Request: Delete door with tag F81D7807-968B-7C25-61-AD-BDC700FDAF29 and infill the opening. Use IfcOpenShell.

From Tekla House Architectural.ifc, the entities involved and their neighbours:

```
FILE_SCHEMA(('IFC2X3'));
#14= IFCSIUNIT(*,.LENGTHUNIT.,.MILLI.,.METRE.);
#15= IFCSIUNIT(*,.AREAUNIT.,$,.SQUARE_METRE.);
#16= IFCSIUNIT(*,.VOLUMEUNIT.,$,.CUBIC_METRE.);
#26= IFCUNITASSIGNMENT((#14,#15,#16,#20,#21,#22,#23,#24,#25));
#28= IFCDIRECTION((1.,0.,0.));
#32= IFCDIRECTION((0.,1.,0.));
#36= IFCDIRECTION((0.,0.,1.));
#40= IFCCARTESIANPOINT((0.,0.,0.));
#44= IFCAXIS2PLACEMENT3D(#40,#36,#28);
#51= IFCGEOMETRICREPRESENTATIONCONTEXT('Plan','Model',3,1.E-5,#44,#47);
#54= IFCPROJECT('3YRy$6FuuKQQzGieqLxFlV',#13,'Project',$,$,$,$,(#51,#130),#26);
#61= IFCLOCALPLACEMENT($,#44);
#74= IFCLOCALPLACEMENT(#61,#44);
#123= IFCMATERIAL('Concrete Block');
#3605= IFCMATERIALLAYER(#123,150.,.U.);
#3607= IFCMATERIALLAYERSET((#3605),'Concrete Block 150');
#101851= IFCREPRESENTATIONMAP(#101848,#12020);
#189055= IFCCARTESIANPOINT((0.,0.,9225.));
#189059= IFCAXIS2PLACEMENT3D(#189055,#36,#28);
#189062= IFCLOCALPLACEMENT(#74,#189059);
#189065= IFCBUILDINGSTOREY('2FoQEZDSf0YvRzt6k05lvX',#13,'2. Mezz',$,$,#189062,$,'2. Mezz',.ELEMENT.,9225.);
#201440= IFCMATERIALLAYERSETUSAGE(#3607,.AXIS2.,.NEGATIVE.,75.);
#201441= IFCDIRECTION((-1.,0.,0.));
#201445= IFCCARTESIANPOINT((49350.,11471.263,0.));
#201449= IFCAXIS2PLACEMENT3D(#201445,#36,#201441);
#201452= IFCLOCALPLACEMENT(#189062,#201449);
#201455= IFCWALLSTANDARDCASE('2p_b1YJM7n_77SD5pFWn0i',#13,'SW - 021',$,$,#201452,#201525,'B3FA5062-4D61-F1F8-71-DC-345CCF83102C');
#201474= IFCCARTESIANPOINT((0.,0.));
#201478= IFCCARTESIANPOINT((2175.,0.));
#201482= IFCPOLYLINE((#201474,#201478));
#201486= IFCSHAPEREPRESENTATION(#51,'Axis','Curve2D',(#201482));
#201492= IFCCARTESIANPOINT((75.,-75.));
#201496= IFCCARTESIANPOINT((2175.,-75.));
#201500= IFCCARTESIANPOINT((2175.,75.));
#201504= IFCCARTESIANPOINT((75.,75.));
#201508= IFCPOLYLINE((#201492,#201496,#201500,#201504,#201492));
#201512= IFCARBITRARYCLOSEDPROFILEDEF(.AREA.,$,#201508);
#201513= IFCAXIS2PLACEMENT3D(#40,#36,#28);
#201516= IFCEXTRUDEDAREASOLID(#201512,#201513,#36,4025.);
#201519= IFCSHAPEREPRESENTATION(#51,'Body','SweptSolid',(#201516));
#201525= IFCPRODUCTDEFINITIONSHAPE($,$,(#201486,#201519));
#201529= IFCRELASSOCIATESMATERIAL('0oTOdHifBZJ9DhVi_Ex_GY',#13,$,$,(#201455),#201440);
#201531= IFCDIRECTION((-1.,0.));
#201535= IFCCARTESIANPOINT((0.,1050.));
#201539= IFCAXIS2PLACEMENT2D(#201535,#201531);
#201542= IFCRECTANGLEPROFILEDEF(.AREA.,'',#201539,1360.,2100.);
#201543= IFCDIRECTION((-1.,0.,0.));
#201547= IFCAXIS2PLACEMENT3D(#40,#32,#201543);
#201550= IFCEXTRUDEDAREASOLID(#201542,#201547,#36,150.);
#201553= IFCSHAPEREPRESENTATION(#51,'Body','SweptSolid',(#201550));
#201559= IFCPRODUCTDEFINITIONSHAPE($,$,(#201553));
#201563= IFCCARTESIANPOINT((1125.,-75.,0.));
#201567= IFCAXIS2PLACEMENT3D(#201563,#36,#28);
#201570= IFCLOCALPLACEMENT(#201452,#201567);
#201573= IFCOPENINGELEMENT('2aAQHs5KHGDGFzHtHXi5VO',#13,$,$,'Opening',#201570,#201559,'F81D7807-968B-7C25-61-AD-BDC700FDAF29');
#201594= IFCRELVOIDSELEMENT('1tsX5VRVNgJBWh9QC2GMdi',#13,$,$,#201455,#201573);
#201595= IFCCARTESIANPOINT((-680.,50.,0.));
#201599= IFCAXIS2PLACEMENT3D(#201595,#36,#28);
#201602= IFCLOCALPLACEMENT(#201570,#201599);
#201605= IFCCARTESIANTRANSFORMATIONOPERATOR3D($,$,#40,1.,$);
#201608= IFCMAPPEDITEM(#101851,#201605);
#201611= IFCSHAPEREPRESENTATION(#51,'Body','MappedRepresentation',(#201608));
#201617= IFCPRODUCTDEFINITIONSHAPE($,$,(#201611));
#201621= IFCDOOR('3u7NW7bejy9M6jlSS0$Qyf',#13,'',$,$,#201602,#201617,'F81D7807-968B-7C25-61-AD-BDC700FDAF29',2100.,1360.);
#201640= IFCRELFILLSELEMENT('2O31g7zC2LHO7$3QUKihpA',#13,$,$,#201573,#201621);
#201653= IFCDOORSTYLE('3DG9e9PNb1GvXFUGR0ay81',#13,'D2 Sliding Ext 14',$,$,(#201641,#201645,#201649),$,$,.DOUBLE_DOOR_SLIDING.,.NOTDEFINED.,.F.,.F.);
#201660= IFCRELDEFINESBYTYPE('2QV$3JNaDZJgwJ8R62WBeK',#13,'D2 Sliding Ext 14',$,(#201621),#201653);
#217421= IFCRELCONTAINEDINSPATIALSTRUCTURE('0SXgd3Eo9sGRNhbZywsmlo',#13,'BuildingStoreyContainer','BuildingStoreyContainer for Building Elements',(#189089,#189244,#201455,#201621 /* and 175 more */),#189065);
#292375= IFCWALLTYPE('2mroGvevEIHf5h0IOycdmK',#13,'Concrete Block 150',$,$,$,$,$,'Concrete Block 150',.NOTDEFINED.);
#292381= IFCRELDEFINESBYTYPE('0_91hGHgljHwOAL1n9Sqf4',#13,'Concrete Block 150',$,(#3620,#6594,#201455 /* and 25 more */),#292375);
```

```python
import ifcopenshell
import ifcopenshell.api.feature
import ifcopenshell.api.root
import ifcopenshell.geom
import ifcopenshell.util.shape

model = ifcopenshell.open("Tekla House Architectural.ifc")
settings = ifcopenshell.geom.settings()


def volume(element):
    """Net volume in cubic metres, openings subtracted."""
    shape = ifcopenshell.geom.create_shape(settings, element)
    return ifcopenshell.util.shape.get_volume(shape.geometry)


door = model.by_guid("3u7NW7bejy9M6jlSS0$Qyf")
opening = door.FillsVoids[0].RelatingOpeningElement
wall = opening.VoidsElements[0].RelatingBuildingElement
before = volume(wall)

ifcopenshell.api.root.remove_product(model, product=door)
ifcopenshell.api.feature.remove_feature(model, feature=opening)

after = volume(wall)

print(f"wall volume {before:.3f} -> {after:.3f} m3")

model.write("Tekla House Architectural_edited.ifc")
```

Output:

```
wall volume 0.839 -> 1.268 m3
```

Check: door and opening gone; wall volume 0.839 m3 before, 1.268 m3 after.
